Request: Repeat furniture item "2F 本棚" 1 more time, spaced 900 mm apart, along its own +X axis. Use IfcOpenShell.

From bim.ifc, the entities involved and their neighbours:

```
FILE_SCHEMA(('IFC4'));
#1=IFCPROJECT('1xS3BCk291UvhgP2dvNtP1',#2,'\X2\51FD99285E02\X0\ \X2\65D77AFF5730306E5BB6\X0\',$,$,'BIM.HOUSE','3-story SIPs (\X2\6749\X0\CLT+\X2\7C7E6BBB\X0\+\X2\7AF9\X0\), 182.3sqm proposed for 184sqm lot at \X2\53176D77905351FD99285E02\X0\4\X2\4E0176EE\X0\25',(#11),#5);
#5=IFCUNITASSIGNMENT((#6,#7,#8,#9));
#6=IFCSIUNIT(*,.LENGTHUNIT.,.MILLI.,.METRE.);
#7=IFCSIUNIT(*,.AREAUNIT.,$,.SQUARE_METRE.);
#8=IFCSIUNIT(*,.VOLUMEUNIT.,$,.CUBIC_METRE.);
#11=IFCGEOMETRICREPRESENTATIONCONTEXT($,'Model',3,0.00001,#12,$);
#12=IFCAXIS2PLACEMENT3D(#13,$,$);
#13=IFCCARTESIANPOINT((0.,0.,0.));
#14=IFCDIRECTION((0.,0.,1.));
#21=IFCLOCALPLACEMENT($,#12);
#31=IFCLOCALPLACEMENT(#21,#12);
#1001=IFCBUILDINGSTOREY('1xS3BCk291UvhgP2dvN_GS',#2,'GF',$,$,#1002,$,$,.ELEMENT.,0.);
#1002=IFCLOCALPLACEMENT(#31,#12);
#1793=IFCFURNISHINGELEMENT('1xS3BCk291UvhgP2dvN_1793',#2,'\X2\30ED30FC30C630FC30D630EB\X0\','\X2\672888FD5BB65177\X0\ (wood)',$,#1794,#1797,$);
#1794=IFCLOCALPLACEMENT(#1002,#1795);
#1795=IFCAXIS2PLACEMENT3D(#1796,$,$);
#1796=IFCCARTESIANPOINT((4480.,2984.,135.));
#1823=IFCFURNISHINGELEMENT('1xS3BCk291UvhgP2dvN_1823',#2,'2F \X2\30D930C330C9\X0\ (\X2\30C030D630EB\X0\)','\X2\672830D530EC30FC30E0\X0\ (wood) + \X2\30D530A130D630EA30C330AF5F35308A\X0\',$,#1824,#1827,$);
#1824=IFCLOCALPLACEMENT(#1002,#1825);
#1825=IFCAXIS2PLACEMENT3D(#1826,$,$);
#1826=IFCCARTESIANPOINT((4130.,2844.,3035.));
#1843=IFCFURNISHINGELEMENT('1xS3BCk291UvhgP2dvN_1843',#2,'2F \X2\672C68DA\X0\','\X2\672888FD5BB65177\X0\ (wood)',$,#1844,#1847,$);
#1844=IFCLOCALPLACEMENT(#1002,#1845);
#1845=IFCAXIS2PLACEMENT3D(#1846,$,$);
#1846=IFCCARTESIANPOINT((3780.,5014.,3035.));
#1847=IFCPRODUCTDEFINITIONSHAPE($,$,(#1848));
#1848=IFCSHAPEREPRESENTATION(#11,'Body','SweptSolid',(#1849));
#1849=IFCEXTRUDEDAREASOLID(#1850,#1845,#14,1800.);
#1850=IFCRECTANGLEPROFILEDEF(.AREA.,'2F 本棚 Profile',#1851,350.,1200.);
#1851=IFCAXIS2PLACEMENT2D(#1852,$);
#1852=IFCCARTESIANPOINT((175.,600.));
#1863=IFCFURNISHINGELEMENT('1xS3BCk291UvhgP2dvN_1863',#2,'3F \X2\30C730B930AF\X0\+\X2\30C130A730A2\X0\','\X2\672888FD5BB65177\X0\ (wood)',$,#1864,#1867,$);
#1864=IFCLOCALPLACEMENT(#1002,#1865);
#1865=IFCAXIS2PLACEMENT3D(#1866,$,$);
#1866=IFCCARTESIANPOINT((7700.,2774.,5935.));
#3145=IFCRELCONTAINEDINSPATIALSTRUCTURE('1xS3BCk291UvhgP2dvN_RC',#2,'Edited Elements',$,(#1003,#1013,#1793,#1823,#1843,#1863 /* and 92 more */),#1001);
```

```python
import ifcopenshell
import ifcopenshell.api.geometry
import ifcopenshell.api.root
import ifcopenshell.util.element
import ifcopenshell.util.placement

model = ifcopenshell.open("bim.ifc")


def reuse_history(source, copy):
    """copy_class also copies each property set's owner history, people and application; keep the originals."""
    for rel in copy.IsDefinedBy:
        if rel.is_a("IfcRelDefinesByProperties") and (history := rel.RelatingPropertyDefinition.OwnerHistory):
            rel.RelatingPropertyDefinition.OwnerHistory = source.OwnerHistory
            ifcopenshell.util.element.remove_deep2(model, history)


source = model.by_id(1843)
base = ifcopenshell.util.placement.get_local_placement(source.ObjectPlacement)
step = base[:3, 0] * 900.0

for i in range(1, 2):
    copy = ifcopenshell.api.root.copy_class(model, product=source)
    copy.Representation = ifcopenshell.util.element.copy_deep(
        model, source.Representation, exclude=["IfcGeometricRepresentationContext", "IfcRepresentationMap"]
    )
    reuse_history(source, copy)
    matrix = base.copy()
    matrix[:3, 3] += i * step
    print("added at", matrix[:3, 3].round(3) + 0.0)
    ifcopenshell.api.geometry.edit_object_placement(model, product=copy, matrix=matrix, is_si=False)

model.write("bim_rev.ifc")
```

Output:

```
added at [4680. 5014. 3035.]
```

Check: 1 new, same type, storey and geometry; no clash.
